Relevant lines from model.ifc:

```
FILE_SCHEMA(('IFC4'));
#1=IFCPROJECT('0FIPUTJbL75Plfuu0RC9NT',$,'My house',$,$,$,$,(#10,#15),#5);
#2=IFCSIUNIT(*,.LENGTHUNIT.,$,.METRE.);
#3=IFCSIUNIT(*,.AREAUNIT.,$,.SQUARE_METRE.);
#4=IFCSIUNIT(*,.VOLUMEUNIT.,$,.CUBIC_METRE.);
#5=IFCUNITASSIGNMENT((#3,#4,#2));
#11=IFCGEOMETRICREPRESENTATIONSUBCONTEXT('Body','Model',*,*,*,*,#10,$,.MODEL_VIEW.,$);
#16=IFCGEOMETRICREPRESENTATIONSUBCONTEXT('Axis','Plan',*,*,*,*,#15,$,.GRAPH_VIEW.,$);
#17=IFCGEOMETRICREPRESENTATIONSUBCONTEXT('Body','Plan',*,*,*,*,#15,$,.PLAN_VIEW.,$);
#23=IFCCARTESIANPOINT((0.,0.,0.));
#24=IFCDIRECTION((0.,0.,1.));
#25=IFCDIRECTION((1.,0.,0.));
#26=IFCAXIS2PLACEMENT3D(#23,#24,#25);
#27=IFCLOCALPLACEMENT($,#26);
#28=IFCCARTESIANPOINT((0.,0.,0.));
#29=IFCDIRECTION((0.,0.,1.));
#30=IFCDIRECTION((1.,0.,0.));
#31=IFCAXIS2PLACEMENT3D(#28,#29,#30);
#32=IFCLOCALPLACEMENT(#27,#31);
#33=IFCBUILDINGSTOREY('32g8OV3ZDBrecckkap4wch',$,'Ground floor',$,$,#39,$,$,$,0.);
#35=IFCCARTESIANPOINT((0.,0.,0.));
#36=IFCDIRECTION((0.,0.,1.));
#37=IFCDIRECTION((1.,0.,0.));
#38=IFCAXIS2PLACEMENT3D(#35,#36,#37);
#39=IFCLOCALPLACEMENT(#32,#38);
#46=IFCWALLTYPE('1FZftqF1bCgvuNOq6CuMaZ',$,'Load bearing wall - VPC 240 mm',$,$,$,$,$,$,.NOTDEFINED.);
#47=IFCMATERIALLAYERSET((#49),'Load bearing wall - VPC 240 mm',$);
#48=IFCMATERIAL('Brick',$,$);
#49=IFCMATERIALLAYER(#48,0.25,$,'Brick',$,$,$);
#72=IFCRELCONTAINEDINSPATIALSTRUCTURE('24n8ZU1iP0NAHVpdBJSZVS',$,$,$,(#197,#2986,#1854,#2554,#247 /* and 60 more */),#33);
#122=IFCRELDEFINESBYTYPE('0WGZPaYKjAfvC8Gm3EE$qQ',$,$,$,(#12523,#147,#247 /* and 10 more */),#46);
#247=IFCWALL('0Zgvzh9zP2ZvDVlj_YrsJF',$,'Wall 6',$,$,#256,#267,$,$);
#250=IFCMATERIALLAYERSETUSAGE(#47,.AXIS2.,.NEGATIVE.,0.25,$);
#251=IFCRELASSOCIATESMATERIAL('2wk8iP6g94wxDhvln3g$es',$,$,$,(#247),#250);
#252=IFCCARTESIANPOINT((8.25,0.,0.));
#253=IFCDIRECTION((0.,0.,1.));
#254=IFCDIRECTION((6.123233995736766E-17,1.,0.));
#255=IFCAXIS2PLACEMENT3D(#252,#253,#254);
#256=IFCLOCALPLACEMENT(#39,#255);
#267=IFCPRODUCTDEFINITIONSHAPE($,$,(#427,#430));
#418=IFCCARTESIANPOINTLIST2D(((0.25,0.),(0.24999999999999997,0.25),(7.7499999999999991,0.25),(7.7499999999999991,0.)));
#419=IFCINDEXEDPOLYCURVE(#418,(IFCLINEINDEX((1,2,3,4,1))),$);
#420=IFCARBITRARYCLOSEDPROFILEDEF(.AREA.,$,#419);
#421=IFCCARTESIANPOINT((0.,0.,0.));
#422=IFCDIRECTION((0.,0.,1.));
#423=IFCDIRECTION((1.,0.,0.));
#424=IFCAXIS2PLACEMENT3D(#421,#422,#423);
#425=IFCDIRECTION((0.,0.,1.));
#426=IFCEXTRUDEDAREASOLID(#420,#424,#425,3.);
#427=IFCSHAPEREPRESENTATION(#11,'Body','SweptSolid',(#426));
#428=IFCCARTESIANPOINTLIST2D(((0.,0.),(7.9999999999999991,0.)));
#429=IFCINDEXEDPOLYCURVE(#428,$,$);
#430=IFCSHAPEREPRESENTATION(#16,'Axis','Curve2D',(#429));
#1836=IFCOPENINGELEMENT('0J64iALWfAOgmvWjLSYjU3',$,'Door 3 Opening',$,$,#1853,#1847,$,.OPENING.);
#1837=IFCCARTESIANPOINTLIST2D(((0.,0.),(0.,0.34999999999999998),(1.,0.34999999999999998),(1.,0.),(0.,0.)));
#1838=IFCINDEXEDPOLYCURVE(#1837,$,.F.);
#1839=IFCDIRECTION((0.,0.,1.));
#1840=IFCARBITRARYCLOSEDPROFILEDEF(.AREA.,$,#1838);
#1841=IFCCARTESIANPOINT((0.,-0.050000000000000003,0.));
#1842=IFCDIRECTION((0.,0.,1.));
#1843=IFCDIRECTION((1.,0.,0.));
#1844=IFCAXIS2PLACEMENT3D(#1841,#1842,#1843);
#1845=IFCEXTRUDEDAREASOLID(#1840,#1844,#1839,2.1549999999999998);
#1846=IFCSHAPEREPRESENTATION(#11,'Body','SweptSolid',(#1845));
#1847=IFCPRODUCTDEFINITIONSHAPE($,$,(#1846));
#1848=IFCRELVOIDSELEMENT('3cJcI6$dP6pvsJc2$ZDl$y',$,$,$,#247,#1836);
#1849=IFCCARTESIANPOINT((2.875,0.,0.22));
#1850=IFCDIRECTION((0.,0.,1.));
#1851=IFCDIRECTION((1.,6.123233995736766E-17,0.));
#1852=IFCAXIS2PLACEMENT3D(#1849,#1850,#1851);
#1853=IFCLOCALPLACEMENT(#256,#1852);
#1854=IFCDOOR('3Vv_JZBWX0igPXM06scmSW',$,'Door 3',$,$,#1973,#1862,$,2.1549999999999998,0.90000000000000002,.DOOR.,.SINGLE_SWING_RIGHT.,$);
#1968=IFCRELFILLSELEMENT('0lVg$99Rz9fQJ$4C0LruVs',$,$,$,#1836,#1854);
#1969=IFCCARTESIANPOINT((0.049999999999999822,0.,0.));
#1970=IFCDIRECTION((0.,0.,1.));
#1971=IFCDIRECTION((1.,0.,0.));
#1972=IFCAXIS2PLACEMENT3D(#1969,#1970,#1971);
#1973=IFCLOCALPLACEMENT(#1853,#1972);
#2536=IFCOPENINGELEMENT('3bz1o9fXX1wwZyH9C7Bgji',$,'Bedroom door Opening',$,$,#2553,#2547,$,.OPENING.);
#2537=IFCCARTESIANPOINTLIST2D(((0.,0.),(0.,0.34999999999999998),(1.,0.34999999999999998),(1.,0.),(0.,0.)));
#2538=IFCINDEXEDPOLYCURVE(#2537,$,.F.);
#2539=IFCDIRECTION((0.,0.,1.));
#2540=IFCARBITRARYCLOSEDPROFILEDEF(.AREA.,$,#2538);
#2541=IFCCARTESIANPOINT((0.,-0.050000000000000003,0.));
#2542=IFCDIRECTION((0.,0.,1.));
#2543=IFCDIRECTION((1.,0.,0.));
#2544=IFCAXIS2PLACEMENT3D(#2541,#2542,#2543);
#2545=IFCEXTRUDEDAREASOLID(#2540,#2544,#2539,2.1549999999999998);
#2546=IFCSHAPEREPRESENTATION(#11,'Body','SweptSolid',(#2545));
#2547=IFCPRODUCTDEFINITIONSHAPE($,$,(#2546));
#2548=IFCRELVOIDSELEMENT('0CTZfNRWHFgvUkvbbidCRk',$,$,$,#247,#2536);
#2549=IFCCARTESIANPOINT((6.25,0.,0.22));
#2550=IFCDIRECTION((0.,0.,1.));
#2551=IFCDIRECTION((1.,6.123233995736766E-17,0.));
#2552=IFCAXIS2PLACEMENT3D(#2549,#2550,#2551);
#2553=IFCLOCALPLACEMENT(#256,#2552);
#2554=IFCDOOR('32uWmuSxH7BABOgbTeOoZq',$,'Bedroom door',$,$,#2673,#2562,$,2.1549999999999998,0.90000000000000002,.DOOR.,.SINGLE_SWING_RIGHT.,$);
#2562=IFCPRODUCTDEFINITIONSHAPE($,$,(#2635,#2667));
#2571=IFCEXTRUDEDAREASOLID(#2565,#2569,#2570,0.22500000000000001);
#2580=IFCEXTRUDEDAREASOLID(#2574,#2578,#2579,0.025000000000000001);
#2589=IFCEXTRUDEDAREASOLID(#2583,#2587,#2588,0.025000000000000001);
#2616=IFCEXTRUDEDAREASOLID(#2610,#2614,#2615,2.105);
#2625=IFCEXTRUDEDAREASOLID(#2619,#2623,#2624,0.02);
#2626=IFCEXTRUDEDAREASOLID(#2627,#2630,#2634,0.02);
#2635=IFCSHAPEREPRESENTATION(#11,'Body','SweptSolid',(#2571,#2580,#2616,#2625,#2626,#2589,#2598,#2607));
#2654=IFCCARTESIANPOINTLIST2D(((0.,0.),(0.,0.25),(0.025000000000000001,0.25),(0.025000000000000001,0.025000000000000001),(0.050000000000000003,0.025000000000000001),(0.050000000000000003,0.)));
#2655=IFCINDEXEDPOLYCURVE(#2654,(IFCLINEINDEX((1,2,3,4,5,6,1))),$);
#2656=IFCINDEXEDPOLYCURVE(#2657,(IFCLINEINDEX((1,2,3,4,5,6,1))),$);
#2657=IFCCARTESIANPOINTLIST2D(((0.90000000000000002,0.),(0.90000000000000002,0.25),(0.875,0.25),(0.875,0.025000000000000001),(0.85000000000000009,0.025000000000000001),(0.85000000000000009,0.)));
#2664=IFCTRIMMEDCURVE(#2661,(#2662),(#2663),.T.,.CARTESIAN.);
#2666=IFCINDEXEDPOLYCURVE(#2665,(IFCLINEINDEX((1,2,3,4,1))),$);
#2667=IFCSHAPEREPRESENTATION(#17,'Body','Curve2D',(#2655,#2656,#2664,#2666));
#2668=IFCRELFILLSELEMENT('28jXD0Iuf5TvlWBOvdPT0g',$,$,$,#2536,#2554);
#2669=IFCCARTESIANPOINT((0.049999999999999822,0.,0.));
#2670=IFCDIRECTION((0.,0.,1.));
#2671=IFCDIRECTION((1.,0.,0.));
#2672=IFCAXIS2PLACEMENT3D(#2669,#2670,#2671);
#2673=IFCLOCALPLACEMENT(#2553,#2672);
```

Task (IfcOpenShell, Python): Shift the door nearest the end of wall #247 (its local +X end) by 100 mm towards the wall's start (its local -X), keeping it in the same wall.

```python
import ifcopenshell
import ifcopenshell.api.geometry
import ifcopenshell.util.placement
import ifcopenshell.util.unit

model = ifcopenshell.open("model.ifc")
unit_scale = ifcopenshell.util.unit.calculate_unit_scale(model)

door = model.by_guid("32uWmuSxH7BABOgbTeOoZq")
opening = door.FillsVoids[0].RelatingOpeningElement
wall = opening.VoidsElements[0].RelatingBuildingElement

wall_matrix = ifcopenshell.util.placement.get_local_placement(wall.ObjectPlacement)
shift = wall_matrix[:3, 0] * -0.1 / unit_scale
before = ifcopenshell.util.placement.get_local_placement(door.ObjectPlacement)[:3, 3].copy()

# The door is placed relative to its opening, so it follows when the opening moves.
matrix = ifcopenshell.util.placement.get_local_placement(opening.ObjectPlacement)
matrix[:3, 3] += shift
ifcopenshell.api.geometry.edit_object_placement(
    model, product=opening, matrix=matrix, is_si=False, should_transform_children=True
)

after = ifcopenshell.util.placement.get_local_placement(door.ObjectPlacement)[:3, 3]
print("door moved by", (after - before).round(3) + 0.0)

model.write("model_updated.ifc")
```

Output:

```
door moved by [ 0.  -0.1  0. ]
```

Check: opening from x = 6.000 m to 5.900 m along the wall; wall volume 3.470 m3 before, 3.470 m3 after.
